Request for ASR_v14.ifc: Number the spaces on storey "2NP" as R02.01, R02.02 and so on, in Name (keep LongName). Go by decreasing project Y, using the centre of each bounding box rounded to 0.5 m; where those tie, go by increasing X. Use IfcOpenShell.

First a look at what the model holds.

```python
import ifcopenshell
import ifcopenshell.util.element
import ifcopenshell.util.placement

model = ifcopenshell.open("ASR_v14.ifc")
print(model.schema)
storey = next(s for s in model.by_type("IfcBuildingStorey") if s.Name == "2NP")
spaces = [e for e in ifcopenshell.util.element.get_decomposition(storey) if e.is_a("IfcSpace")]
for e in sorted(spaces, key=lambda e: e.id()):
    origin = ifcopenshell.util.placement.get_local_placement(e.ObjectPlacement)[:3, 3]
    print(e.id(), e.Name, e.LongName, origin.round(2) + 0.0, sep=" | ")
```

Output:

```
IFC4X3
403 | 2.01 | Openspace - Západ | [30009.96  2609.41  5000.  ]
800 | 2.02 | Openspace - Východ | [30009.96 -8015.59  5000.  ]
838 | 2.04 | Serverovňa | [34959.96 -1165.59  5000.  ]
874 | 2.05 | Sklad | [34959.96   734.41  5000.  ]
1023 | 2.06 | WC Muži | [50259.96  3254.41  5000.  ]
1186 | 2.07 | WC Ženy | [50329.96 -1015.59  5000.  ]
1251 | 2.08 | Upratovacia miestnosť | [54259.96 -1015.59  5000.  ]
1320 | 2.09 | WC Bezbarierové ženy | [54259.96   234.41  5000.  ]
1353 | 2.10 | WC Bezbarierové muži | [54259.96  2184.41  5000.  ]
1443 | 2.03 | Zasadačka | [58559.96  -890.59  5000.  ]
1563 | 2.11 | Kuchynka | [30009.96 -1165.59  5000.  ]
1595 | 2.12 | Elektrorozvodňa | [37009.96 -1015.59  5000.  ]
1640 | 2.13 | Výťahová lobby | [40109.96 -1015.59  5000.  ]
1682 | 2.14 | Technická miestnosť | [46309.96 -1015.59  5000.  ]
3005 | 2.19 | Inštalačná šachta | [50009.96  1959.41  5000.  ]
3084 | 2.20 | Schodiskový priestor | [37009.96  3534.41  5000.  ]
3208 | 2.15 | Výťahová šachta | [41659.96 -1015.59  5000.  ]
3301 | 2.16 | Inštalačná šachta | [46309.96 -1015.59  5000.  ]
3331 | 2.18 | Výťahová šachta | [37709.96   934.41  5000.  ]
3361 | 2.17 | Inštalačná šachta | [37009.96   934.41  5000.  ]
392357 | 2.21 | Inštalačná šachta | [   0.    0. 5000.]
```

```python
import ifcopenshell
import ifcopenshell.geom
import ifcopenshell.util.element
import ifcopenshell.util.shape

model = ifcopenshell.open("ASR_v14.ifc")
settings = ifcopenshell.geom.settings()
settings.set("use-world-coords", True)


def centre(element):
    shape = ifcopenshell.geom.create_shape(settings, element)
    return ifcopenshell.util.shape.get_bbox_centroid(shape.geometry)


storey = next(s for s in model.by_type("IfcBuildingStorey") if s.Name == "2NP")
spaces = [e for e in ifcopenshell.util.element.get_decomposition(storey) if e.is_a("IfcSpace")]

# Insertion points can sit at a corner or the storey origin, so sort by the geometry (in metres).
centres = {e: centre(e) for e in spaces}
spaces.sort(key=lambda e: (-round(centres[e][1] / 0.5), centres[e][0]))

for i, e in enumerate(spaces, start=1):
    number = f"R02.{i:02d}"
    e.Name = number
    print(e.id(), number)

model.write("ASR_v14-out.ifc")
```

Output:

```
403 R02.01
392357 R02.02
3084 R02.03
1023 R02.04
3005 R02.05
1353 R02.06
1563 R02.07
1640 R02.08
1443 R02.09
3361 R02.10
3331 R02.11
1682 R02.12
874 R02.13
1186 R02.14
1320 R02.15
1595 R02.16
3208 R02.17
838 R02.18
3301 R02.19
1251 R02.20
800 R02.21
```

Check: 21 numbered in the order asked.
